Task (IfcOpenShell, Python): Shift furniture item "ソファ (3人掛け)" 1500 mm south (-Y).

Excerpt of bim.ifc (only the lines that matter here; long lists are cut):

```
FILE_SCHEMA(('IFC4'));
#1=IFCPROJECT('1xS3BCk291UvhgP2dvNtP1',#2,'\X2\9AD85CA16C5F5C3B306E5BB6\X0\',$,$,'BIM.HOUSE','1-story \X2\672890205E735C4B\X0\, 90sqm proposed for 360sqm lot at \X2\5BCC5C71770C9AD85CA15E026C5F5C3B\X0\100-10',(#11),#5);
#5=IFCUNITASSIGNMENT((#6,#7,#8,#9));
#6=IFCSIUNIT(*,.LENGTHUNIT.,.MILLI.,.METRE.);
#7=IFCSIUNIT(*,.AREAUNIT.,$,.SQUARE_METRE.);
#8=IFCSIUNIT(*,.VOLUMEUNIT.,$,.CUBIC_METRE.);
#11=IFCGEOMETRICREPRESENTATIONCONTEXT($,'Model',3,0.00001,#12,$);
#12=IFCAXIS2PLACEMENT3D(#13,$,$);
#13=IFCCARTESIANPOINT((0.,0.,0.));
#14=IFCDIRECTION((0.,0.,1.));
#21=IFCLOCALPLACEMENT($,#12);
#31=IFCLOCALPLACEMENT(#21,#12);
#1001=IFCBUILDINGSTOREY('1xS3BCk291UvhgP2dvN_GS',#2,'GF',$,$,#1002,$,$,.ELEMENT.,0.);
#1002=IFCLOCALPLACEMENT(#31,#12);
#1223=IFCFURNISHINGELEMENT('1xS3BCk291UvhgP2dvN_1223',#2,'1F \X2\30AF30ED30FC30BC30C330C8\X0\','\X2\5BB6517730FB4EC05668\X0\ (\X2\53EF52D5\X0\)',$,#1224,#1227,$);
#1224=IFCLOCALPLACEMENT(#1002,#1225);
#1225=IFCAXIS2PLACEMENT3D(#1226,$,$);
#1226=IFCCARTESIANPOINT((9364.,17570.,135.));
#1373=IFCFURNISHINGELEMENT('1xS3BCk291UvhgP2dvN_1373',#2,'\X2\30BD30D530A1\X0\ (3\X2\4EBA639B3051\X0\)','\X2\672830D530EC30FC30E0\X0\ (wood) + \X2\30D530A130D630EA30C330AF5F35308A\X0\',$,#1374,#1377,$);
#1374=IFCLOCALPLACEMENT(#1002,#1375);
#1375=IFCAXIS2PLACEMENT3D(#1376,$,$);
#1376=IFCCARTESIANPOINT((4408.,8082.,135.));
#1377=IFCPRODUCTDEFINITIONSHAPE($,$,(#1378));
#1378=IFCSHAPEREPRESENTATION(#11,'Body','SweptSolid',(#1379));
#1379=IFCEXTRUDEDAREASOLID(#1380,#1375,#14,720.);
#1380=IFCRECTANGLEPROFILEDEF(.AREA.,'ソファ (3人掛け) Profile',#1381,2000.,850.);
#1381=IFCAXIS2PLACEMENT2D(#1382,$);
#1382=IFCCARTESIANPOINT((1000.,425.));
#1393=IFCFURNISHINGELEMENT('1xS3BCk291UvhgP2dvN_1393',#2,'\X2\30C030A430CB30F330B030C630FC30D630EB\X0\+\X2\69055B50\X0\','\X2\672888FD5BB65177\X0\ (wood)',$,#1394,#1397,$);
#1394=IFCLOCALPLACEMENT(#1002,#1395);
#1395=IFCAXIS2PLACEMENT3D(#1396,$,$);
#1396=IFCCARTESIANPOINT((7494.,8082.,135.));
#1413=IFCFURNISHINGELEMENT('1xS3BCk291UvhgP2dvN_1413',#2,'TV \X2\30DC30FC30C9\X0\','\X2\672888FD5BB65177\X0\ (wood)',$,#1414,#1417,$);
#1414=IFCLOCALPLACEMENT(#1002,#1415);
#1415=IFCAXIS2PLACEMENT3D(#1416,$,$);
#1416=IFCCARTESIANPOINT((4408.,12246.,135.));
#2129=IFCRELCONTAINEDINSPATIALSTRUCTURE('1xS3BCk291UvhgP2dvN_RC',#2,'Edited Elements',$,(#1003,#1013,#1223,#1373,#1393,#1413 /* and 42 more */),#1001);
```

```python
import ifcopenshell
import ifcopenshell.api.geometry
import ifcopenshell.util.placement

model = ifcopenshell.open("bim.ifc")

item = model.by_id(1373)
matrix = ifcopenshell.util.placement.get_local_placement(item.ObjectPlacement)
matrix[1, 3] -= 1500.0
ifcopenshell.api.geometry.edit_object_placement(model, product=item, matrix=matrix, is_si=False)

print(ifcopenshell.util.placement.get_local_placement(item.ObjectPlacement).round(3) + 0.0)

model.write("bim_edited.ifc")
```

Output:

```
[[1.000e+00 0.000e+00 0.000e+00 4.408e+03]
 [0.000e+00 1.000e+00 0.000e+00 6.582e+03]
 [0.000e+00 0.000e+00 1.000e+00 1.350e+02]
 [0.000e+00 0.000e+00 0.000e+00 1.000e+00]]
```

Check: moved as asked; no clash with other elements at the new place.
